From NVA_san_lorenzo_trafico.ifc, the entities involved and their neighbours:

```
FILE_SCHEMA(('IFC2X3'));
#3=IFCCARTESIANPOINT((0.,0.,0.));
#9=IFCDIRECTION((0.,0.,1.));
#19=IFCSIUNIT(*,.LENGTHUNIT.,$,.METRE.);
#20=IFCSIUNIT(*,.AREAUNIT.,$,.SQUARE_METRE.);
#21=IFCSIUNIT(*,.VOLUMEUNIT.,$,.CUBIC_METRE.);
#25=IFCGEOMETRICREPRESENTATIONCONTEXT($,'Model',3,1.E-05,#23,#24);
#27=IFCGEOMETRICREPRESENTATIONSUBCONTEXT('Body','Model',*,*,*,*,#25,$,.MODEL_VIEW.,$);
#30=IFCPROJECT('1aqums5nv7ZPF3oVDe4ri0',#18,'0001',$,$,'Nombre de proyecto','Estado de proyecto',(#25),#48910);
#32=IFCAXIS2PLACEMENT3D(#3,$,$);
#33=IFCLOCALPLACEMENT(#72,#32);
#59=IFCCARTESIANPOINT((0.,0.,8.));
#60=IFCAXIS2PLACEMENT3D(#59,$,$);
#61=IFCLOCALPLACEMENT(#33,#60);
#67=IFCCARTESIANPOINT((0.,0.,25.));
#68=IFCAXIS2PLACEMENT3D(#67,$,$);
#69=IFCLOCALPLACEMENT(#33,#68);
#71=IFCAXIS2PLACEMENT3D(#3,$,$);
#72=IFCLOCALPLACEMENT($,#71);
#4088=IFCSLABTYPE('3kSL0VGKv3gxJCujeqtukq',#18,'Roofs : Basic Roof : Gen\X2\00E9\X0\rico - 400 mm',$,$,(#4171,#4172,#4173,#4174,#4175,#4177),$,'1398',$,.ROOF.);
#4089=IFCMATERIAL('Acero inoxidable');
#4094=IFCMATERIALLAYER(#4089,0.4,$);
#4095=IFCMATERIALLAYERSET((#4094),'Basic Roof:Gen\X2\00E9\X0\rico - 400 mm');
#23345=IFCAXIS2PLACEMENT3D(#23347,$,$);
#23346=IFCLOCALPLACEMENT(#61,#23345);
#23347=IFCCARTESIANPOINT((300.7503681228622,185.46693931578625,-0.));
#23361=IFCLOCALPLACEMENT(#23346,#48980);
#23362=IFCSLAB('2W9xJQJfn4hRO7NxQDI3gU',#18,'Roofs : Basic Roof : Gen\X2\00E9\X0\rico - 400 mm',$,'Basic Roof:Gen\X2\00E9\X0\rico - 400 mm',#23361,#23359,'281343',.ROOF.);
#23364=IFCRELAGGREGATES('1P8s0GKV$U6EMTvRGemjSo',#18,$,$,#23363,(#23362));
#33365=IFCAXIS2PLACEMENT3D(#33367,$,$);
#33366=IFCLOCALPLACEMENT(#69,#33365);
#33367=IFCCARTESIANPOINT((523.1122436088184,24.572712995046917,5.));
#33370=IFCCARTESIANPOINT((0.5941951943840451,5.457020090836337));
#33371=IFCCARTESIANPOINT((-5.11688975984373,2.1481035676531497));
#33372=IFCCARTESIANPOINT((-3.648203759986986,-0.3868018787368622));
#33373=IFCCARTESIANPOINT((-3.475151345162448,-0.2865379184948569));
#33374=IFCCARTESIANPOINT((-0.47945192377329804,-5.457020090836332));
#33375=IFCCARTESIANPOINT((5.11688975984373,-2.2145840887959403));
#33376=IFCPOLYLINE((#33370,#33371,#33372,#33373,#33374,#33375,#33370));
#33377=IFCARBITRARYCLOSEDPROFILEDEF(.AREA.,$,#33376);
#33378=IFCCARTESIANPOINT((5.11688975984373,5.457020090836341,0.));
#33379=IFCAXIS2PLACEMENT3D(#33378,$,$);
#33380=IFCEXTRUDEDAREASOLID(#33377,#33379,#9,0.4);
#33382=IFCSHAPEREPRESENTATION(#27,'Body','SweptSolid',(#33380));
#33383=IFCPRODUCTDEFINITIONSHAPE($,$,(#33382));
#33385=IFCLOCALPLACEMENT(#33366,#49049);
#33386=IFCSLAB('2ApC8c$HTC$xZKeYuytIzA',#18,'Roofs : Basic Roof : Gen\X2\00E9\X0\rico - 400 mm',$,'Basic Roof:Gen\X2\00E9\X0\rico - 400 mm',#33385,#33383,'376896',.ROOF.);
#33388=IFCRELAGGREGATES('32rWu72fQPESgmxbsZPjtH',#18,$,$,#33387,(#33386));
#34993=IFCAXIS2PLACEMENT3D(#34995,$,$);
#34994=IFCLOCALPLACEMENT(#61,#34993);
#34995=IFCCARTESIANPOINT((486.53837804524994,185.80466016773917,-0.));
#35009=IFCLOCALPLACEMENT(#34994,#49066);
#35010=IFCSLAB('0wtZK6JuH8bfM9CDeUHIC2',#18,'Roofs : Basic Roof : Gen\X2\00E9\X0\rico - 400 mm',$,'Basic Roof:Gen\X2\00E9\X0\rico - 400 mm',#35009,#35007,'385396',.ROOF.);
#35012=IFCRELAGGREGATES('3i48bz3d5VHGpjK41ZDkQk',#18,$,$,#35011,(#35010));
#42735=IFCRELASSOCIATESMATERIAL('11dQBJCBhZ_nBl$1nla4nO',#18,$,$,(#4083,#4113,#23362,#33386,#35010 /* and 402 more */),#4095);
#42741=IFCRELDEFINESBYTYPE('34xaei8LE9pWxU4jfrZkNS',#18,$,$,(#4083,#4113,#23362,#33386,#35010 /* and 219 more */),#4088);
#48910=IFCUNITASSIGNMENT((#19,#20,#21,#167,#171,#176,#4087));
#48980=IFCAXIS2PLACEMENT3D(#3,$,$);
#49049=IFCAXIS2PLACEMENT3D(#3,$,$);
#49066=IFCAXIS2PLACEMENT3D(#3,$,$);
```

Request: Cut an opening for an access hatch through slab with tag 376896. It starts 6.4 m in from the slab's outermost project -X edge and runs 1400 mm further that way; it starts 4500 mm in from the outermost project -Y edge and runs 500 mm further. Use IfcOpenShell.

```python
import numpy as np
import ifcopenshell
import ifcopenshell.api.feature
import ifcopenshell.api.geometry
import ifcopenshell.api.root
import ifcopenshell.geom
import ifcopenshell.util.placement
import ifcopenshell.util.representation
import ifcopenshell.util.shape
import ifcopenshell.util.unit

model = ifcopenshell.open("NVA_san_lorenzo_trafico.ifc")
unit_scale = ifcopenshell.util.unit.calculate_unit_scale(model)
settings = ifcopenshell.geom.settings()


def volume(element):
    """Net volume in cubic metres, openings subtracted."""
    shape = ifcopenshell.geom.create_shape(settings, element)
    return ifcopenshell.util.shape.get_volume(shape.geometry)


slab = model.by_guid("2ApC8c$HTC$xZKeYuytIzA")
before = volume(slab)

# Extent in the slab's own axes, in metres. The edges named are its -X and -Y sides.
slab_shape = ifcopenshell.geom.create_shape(settings, slab)
vertices = ifcopenshell.util.shape.get_vertices(slab_shape.geometry)
x_min, y_min, bottom = vertices.min(axis=0)
top = vertices[:, 2].max()

opening = ifcopenshell.api.root.create_entity(model, ifc_class="IfcOpeningElement", name="Access hatch opening")
context = ifcopenshell.util.representation.get_context(model, "Model", "Body", "MODEL_VIEW")
width, depth = 1.4, 0.5
outline = [(0.0, 0.0), (width, 0.0), (width, depth), (0.0, depth), (0.0, 0.0)]
# Overshoot both faces by 50 mm so the cut is clean.
shape = ifcopenshell.api.geometry.add_slab_representation(
    model, context=context, depth=top - bottom + 0.1, polyline=outline
)
ifcopenshell.api.geometry.assign_representation(model, product=opening, representation=shape)

matrix = ifcopenshell.util.placement.get_local_placement(slab.ObjectPlacement)
matrix[:, 3] = matrix @ np.append(np.array([x_min + 6.4, y_min + 4.5, bottom - 0.05]) / unit_scale, 1.0)
ifcopenshell.api.geometry.edit_object_placement(model, product=opening, matrix=matrix, is_si=False)
ifcopenshell.api.feature.add_feature(model, feature=opening, element=slab)

after = volume(slab)

print(f"slab volume {before:.3f} -> {after:.3f} m3")

model.write("NVA_san_lorenzo_trafico_rev.ifc")
```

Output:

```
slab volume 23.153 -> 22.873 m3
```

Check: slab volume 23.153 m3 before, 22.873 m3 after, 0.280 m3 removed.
